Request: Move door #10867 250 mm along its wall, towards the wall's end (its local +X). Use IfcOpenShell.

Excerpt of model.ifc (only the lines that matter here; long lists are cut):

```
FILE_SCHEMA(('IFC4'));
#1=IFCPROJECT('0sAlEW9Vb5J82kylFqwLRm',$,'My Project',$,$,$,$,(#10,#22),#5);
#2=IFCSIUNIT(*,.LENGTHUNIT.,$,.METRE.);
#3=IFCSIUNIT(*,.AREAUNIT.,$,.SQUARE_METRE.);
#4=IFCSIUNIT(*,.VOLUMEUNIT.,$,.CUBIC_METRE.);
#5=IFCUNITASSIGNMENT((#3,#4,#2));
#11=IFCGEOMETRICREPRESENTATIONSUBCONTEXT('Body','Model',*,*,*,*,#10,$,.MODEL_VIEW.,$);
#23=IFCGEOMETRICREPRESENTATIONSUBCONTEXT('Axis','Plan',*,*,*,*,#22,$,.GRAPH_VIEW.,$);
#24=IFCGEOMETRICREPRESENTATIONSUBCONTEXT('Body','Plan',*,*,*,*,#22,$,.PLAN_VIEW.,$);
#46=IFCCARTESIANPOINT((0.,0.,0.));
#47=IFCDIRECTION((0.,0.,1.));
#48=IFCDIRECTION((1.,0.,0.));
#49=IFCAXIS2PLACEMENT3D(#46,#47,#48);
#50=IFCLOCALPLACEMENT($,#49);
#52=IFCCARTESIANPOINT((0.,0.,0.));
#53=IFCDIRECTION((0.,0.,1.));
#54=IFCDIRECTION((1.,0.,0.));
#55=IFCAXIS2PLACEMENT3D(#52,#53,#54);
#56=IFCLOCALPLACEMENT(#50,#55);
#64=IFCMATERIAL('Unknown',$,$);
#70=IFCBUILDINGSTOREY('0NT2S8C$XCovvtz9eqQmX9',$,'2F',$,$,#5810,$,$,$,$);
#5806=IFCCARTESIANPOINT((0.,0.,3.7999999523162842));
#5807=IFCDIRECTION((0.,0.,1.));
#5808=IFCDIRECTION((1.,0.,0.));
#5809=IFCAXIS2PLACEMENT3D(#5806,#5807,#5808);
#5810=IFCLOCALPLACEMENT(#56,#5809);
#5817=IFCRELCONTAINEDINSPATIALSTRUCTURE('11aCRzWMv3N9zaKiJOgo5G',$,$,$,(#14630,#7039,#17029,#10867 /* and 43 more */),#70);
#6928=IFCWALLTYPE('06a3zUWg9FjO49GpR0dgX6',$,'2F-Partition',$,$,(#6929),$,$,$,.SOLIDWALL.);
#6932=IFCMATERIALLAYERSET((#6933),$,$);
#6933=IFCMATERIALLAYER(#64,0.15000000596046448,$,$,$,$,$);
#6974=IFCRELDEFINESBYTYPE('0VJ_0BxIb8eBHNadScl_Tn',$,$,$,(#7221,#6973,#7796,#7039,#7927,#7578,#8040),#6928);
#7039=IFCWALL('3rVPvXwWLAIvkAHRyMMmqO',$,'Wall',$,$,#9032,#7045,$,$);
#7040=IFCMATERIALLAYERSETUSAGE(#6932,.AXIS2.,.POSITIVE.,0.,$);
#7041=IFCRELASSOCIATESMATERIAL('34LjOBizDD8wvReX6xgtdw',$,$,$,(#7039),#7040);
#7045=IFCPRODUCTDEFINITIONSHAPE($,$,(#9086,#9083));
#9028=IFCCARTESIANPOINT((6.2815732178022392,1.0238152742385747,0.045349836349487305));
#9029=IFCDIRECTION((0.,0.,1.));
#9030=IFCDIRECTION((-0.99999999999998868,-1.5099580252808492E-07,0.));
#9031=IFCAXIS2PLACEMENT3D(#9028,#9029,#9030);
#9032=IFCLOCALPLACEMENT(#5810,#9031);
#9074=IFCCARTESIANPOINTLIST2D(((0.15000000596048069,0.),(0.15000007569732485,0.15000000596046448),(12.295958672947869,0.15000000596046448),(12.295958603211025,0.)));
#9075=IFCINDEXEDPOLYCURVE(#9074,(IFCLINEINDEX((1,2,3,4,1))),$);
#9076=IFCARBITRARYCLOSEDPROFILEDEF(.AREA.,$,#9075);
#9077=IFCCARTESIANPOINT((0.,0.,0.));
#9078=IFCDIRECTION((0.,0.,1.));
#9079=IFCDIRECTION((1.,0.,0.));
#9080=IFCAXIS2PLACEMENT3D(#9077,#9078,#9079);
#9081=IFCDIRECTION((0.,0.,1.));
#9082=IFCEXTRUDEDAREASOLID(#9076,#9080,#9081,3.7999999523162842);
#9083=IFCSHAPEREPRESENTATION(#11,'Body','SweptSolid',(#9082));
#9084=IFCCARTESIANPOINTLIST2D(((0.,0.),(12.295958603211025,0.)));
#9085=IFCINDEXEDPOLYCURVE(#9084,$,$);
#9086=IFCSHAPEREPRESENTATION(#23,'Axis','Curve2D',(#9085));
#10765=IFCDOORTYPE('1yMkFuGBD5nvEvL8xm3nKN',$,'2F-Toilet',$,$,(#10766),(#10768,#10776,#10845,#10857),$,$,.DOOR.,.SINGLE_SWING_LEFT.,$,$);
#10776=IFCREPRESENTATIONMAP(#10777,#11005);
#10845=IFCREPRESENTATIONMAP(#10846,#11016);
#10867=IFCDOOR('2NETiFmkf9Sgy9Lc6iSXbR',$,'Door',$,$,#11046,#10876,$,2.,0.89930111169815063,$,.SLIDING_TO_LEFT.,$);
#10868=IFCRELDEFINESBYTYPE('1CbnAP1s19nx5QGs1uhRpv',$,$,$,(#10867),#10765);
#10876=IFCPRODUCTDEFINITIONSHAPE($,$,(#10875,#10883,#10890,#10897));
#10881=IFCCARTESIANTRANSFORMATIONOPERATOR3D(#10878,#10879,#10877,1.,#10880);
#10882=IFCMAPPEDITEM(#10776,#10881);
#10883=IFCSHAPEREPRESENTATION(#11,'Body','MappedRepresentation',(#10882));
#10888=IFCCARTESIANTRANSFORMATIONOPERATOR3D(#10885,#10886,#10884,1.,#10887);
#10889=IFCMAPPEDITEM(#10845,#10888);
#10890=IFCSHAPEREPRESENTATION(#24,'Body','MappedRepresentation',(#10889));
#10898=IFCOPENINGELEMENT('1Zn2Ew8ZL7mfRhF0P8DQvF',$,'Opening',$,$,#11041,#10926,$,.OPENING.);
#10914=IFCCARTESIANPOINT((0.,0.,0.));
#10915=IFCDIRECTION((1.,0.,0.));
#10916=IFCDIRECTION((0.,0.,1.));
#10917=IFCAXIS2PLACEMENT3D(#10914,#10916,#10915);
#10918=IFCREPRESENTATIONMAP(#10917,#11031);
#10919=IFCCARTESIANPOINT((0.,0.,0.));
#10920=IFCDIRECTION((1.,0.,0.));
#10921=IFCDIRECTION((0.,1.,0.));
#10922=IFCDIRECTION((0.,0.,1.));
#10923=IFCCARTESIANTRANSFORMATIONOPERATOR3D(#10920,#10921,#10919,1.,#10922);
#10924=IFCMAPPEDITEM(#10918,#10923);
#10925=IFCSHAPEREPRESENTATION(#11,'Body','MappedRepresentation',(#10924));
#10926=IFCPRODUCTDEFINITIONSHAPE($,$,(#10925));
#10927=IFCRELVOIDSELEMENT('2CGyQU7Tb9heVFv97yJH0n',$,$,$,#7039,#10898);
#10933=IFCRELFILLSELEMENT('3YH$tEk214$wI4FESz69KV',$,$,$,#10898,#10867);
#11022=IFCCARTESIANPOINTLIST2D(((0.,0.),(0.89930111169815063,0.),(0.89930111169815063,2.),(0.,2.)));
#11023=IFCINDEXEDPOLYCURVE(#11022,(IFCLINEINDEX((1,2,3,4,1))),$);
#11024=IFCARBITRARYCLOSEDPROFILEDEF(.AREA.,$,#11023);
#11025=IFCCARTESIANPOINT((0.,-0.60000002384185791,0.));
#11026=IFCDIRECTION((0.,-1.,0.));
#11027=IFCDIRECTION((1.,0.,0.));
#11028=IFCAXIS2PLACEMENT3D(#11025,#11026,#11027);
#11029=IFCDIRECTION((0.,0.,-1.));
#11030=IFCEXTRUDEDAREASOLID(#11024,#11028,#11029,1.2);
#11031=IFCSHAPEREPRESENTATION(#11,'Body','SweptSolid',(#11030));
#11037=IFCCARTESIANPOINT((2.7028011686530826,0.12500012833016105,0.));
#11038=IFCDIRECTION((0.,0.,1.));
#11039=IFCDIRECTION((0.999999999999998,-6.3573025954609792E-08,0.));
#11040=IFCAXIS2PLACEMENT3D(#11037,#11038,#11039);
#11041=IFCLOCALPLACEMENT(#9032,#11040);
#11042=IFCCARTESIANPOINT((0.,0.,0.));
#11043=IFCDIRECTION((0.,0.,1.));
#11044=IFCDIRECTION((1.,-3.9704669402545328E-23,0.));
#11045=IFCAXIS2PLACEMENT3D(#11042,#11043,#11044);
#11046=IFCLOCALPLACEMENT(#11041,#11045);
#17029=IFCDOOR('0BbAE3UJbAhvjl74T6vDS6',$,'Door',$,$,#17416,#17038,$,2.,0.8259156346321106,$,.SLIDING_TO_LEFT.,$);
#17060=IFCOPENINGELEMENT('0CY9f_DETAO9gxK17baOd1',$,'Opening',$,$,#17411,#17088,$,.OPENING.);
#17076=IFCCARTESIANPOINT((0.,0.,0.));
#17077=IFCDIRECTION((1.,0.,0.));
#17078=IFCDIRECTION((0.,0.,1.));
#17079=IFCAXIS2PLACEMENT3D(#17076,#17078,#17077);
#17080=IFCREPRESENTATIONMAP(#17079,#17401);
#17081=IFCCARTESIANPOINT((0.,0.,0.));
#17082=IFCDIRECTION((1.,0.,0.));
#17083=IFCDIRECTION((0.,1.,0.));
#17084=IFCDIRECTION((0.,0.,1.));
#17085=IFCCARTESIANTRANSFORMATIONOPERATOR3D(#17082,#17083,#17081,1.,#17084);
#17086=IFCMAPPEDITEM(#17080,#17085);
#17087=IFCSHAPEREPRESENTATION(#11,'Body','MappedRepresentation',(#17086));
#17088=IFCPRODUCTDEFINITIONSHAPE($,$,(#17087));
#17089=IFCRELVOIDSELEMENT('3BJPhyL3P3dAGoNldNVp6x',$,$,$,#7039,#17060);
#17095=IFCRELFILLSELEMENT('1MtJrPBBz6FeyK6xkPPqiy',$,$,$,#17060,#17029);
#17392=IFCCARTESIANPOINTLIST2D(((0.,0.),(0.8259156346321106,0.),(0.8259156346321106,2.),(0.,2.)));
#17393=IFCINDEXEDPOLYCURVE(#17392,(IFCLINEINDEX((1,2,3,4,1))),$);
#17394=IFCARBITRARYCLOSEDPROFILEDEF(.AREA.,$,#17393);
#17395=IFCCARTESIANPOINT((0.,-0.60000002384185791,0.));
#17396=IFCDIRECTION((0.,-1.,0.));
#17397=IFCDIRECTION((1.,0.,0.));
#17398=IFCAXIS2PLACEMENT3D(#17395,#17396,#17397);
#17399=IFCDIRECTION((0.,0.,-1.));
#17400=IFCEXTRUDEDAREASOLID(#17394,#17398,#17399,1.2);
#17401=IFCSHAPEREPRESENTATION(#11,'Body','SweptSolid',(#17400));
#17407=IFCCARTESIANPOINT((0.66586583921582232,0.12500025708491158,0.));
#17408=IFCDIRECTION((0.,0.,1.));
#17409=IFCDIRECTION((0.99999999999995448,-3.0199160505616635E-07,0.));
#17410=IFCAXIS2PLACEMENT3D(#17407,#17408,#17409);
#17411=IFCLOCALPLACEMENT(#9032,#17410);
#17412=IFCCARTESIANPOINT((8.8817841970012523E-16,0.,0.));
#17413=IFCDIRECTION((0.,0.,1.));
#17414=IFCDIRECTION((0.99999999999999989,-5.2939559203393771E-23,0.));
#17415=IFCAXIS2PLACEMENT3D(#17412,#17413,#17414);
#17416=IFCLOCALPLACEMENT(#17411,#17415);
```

```python
import ifcopenshell
import ifcopenshell.api.geometry
import ifcopenshell.util.placement
import ifcopenshell.util.unit

model = ifcopenshell.open("model.ifc")
unit_scale = ifcopenshell.util.unit.calculate_unit_scale(model)

door = model.by_guid("2NETiFmkf9Sgy9Lc6iSXbR")
opening = door.FillsVoids[0].RelatingOpeningElement
wall = opening.VoidsElements[0].RelatingBuildingElement

wall_matrix = ifcopenshell.util.placement.get_local_placement(wall.ObjectPlacement)
shift = wall_matrix[:3, 0] * 0.25 / unit_scale
before = ifcopenshell.util.placement.get_local_placement(door.ObjectPlacement)[:3, 3].copy()

# The door is placed relative to its opening, so it follows when the opening moves.
matrix = ifcopenshell.util.placement.get_local_placement(opening.ObjectPlacement)
matrix[:3, 3] += shift
ifcopenshell.api.geometry.edit_object_placement(
    model, product=opening, matrix=matrix, is_si=False, should_transform_children=True
)

after = ifcopenshell.util.placement.get_local_placement(door.ObjectPlacement)[:3, 3]
print("door moved by", (after - before).round(3) + 0.0)

model.write("model-out.ifc")
```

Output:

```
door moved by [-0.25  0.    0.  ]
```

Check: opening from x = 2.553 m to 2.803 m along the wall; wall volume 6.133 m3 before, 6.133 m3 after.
